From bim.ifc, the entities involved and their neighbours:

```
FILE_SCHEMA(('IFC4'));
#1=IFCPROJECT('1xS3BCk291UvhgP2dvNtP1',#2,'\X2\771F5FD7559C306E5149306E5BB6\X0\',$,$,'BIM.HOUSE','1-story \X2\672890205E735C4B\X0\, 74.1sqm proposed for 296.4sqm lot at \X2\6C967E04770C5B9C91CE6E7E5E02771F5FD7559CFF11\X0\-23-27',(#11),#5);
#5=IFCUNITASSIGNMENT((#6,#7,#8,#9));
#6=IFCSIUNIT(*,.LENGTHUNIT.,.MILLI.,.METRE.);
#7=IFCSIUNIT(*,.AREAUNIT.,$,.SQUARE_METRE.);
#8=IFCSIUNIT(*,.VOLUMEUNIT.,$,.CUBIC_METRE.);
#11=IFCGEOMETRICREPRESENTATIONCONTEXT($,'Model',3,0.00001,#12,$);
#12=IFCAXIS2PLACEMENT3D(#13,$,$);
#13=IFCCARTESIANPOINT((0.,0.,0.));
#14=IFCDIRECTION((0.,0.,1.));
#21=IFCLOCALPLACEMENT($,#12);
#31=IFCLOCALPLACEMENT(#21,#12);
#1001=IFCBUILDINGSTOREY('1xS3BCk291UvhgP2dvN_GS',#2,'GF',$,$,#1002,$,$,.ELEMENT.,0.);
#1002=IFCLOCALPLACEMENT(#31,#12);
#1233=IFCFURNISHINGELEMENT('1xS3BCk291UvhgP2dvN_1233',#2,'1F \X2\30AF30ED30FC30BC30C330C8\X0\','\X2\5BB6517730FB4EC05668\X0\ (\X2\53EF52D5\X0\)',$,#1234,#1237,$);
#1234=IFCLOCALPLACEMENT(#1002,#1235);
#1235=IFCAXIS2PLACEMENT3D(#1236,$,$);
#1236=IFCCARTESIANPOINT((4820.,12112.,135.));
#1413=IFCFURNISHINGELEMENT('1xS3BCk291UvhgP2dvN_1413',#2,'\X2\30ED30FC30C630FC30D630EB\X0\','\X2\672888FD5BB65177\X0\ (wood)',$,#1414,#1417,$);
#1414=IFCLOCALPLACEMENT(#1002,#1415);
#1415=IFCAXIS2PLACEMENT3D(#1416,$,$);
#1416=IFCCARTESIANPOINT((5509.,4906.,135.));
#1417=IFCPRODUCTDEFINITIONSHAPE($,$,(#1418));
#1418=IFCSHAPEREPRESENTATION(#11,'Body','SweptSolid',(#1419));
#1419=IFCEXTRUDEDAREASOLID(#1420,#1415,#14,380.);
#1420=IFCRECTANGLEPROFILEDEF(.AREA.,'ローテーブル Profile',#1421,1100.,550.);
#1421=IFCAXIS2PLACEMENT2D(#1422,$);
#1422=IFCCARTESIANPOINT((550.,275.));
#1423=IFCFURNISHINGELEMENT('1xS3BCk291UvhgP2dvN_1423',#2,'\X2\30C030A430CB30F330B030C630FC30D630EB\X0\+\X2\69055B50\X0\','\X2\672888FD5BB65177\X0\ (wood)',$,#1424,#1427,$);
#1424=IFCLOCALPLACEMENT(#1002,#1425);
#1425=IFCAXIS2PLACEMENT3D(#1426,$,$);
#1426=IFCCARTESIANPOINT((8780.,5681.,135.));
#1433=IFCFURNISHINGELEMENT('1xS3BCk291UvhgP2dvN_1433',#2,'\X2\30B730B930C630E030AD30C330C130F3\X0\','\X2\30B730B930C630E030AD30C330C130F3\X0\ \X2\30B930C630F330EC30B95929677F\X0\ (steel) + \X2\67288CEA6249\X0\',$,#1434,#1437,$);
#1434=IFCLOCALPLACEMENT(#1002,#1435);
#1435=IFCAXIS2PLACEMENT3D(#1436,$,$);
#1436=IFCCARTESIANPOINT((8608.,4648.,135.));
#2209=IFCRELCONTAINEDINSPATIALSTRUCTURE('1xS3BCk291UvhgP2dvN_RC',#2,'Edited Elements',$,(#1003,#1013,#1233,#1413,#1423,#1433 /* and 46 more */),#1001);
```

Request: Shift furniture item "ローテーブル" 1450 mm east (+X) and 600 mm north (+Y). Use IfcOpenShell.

```python
import ifcopenshell
import ifcopenshell.api.geometry
import ifcopenshell.util.placement
import ifcopenshell.util.unit

model = ifcopenshell.open("bim.ifc")
unit_scale = ifcopenshell.util.unit.calculate_unit_scale(model)

item = model.by_guid("1xS3BCk291UvhgP2dvN_1413")
matrix = ifcopenshell.util.placement.get_local_placement(item.ObjectPlacement)
matrix[0, 3] += 1.45 / unit_scale
matrix[1, 3] += 0.6 / unit_scale
ifcopenshell.api.geometry.edit_object_placement(model, product=item, matrix=matrix, is_si=False)

print(ifcopenshell.util.placement.get_local_placement(item.ObjectPlacement).round(3) + 0.0)

model.write("bim_edited.ifc")
```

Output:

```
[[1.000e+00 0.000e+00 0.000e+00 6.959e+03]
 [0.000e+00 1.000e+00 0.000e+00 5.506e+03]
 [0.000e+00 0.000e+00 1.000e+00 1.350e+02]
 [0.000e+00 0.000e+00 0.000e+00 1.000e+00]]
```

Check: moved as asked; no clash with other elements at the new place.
